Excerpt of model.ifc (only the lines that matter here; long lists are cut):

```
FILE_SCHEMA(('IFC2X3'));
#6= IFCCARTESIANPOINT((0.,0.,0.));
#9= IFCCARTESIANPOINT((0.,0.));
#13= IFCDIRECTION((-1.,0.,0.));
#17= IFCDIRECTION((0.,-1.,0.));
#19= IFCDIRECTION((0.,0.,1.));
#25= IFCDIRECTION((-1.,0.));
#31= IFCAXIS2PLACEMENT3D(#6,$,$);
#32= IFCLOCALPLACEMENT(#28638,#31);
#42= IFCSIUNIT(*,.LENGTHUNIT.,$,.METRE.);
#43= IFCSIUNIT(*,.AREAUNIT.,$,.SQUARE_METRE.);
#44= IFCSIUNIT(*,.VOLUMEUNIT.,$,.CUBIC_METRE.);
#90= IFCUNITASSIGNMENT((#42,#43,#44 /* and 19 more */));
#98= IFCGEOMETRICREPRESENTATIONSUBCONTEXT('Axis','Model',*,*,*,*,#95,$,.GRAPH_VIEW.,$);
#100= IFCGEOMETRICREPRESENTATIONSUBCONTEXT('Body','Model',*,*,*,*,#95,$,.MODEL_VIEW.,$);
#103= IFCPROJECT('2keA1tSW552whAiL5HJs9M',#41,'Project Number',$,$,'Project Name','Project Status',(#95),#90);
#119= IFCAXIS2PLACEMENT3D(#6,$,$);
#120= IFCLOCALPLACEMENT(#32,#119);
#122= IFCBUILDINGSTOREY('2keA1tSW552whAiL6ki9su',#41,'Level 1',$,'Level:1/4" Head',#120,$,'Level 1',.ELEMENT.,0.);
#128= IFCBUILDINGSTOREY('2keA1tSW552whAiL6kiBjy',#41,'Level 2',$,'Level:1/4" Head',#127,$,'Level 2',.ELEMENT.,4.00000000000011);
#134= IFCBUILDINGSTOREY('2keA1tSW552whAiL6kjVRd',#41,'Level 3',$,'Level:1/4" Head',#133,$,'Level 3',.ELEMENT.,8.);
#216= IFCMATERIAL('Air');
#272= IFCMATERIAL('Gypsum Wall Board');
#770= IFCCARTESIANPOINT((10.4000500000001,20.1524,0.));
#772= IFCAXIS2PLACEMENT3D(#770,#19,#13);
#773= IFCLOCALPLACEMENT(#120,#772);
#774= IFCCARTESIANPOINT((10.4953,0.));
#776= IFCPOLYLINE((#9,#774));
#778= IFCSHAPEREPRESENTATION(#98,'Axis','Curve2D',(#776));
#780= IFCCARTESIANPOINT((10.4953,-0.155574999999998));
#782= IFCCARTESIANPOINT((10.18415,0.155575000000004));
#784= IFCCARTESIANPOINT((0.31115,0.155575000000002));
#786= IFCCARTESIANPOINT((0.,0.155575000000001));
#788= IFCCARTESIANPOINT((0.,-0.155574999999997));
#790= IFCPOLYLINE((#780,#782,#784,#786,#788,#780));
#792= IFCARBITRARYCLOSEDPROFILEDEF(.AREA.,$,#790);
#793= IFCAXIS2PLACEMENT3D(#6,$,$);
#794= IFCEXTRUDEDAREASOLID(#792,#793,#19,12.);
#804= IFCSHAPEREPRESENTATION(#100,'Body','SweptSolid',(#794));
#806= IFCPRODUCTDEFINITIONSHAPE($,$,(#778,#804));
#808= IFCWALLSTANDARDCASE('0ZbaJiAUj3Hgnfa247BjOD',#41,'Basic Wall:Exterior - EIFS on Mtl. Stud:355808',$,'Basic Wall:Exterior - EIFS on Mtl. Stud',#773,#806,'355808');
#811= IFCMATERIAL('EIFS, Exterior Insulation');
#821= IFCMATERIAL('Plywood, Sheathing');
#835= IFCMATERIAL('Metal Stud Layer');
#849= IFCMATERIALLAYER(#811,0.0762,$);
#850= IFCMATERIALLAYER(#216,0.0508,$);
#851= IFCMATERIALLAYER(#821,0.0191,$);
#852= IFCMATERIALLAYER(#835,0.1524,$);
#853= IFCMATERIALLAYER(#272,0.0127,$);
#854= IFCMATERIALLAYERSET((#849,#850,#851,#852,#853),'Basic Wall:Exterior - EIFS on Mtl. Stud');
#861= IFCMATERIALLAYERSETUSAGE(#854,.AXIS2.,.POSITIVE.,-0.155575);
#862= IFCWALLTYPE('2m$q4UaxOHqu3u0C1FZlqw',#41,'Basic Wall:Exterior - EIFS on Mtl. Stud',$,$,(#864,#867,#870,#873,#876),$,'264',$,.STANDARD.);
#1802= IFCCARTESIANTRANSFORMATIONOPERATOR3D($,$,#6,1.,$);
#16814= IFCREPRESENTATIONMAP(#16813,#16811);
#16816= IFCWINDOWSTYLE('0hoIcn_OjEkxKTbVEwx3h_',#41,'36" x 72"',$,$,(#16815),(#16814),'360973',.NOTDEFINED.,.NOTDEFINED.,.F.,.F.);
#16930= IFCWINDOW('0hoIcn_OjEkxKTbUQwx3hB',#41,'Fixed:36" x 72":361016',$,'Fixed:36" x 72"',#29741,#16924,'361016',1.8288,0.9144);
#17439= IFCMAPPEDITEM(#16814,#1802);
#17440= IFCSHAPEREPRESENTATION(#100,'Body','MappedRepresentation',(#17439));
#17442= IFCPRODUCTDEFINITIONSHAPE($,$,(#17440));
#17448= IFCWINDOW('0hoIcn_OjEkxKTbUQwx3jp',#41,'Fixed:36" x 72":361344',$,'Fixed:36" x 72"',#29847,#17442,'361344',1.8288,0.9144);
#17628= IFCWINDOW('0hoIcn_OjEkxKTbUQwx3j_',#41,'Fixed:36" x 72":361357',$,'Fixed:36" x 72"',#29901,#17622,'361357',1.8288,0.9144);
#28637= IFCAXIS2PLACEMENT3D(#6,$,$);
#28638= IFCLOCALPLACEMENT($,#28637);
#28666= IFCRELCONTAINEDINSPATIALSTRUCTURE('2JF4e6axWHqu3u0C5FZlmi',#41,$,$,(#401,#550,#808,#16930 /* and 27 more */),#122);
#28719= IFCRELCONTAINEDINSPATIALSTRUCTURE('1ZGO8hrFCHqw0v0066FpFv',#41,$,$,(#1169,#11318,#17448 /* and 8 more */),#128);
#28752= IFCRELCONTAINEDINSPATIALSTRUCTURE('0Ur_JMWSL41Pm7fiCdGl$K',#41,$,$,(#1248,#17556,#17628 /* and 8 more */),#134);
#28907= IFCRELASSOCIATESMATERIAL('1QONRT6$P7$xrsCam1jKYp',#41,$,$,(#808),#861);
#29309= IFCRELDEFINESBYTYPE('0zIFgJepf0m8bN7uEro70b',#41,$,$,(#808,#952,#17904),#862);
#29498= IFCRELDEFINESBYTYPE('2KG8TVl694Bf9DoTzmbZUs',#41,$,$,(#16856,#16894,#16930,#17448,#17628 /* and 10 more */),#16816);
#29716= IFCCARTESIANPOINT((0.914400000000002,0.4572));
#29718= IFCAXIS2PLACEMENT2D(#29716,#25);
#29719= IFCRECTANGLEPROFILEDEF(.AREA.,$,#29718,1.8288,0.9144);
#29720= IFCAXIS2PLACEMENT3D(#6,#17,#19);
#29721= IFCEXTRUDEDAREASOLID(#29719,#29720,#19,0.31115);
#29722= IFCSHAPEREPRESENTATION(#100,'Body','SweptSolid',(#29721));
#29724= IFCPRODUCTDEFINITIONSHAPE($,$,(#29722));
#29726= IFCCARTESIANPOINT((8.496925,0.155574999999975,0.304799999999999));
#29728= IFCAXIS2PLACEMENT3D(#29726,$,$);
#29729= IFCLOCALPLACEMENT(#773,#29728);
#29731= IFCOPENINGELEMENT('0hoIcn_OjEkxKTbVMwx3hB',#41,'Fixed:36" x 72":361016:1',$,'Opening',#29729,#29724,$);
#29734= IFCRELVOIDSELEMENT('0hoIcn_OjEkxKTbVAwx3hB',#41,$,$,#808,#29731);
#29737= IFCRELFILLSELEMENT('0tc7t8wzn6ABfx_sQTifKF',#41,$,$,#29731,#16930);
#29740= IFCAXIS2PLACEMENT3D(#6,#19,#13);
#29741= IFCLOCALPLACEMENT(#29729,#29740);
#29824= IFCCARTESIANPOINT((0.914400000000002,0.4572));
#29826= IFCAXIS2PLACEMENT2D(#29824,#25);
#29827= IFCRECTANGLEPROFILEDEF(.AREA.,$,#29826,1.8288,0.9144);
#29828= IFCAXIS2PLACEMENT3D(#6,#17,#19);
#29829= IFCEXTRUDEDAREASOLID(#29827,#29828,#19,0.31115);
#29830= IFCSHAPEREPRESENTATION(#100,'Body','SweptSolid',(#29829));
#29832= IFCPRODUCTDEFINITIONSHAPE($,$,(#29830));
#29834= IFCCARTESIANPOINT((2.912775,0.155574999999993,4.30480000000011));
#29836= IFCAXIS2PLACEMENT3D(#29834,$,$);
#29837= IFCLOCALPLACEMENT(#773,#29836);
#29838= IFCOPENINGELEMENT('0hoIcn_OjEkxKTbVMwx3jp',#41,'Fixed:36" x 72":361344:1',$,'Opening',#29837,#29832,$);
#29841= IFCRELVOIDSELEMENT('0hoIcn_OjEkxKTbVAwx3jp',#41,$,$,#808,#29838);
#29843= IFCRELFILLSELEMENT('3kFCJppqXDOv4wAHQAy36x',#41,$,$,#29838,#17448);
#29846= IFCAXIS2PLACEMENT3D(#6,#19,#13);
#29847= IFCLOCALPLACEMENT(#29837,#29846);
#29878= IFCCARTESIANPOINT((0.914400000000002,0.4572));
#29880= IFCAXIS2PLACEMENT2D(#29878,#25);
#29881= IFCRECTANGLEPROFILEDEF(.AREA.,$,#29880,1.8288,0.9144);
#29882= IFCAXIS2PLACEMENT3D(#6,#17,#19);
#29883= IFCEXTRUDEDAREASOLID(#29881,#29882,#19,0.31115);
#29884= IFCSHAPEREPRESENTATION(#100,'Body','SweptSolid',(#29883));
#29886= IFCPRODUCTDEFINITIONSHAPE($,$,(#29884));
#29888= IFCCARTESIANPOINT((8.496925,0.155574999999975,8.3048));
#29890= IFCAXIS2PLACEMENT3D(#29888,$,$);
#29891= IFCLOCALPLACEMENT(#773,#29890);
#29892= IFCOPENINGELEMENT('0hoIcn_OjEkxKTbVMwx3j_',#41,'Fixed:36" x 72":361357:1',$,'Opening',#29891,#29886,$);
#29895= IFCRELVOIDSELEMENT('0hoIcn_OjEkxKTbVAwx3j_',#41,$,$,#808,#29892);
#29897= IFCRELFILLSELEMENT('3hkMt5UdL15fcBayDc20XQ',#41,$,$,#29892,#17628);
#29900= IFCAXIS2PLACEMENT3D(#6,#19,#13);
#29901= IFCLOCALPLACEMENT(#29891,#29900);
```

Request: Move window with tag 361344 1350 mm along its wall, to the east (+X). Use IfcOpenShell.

```python
import ifcopenshell
import ifcopenshell.api.geometry
import ifcopenshell.util.placement

model = ifcopenshell.open("model.ifc")

window = model.by_guid("0hoIcn_OjEkxKTbUQwx3jp")
opening = window.FillsVoids[0].RelatingOpeningElement
wall = opening.VoidsElements[0].RelatingBuildingElement

wall_matrix = ifcopenshell.util.placement.get_local_placement(wall.ObjectPlacement)
shift = wall_matrix[:3, 0] * -1.35
before = ifcopenshell.util.placement.get_local_placement(window.ObjectPlacement)[:3, 3].copy()

# The window is placed relative to its opening, so it follows when the opening moves.
matrix = ifcopenshell.util.placement.get_local_placement(opening.ObjectPlacement)
matrix[:3, 3] += shift
ifcopenshell.api.geometry.edit_object_placement(
    model, product=opening, matrix=matrix, is_si=False, should_transform_children=True
)

after = ifcopenshell.util.placement.get_local_placement(window.ObjectPlacement)[:3, 3]
print("window moved by", (after - before).round(3) + 0.0)

model.write("model_v2.ifc")
```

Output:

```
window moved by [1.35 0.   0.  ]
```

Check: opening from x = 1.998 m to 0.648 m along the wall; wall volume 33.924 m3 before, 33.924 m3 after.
